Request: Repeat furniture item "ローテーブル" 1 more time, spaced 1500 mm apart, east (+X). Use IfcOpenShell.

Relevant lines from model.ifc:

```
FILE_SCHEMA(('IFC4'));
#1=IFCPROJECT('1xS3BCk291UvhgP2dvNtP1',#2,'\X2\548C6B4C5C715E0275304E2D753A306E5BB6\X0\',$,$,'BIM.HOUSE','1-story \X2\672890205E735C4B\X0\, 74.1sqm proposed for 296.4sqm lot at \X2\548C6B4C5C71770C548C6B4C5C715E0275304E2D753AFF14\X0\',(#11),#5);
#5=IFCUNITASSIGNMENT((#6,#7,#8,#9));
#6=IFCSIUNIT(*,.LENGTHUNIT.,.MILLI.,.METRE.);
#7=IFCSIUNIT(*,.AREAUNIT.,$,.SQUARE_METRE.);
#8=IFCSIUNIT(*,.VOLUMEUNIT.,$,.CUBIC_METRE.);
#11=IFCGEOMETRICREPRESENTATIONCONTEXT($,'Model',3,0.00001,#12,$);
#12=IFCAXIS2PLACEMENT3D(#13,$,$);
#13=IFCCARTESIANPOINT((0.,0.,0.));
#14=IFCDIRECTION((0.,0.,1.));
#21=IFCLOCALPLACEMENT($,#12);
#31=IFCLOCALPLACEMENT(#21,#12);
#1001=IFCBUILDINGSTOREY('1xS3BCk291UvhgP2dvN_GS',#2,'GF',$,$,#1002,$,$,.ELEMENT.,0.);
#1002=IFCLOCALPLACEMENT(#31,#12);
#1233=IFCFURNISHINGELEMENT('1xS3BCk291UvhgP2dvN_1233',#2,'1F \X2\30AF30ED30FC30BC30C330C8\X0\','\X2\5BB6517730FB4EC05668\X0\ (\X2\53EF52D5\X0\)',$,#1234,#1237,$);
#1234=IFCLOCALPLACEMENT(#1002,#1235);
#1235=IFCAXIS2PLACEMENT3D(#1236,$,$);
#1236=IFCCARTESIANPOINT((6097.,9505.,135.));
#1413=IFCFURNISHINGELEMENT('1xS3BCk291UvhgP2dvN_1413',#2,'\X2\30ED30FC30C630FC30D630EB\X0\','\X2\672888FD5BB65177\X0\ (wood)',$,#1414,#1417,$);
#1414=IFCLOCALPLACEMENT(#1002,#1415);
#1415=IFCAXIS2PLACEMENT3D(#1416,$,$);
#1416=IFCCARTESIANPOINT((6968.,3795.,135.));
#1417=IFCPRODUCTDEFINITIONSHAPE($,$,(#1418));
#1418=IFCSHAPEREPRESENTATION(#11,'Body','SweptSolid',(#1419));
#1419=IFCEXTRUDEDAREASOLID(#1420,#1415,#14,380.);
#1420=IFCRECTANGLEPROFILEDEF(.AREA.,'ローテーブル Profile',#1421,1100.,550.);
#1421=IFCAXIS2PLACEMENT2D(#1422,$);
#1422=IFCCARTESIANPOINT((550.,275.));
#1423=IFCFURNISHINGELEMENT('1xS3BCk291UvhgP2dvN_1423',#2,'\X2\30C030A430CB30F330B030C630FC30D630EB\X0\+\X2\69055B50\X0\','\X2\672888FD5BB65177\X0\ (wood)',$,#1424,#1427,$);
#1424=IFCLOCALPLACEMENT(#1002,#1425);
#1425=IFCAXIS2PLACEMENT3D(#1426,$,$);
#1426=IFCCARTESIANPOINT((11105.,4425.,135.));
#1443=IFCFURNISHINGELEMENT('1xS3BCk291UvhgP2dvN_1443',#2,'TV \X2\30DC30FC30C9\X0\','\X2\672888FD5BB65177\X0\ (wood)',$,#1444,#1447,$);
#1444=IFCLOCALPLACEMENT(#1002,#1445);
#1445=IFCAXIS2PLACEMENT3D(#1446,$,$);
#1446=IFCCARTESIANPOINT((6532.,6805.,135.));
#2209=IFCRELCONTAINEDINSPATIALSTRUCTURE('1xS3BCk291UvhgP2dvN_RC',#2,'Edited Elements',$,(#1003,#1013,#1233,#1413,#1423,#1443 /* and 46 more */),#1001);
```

```python
import numpy as np
import ifcopenshell
import ifcopenshell.api.geometry
import ifcopenshell.api.root
import ifcopenshell.util.element
import ifcopenshell.util.placement
import ifcopenshell.util.unit

model = ifcopenshell.open("model.ifc")
unit_scale = ifcopenshell.util.unit.calculate_unit_scale(model)


def reuse_history(source, copy):
    """copy_class also copies each property set's owner history, people and application; keep the originals."""
    for rel in copy.IsDefinedBy:
        if rel.is_a("IfcRelDefinesByProperties") and (history := rel.RelatingPropertyDefinition.OwnerHistory):
            rel.RelatingPropertyDefinition.OwnerHistory = source.OwnerHistory
            ifcopenshell.util.element.remove_deep2(model, history)


source = model.by_guid("1xS3BCk291UvhgP2dvN_1413")
base = ifcopenshell.util.placement.get_local_placement(source.ObjectPlacement)
step = np.array([1.0, 0.0, 0.0]) * 1.5 / unit_scale

for i in range(1, 2):
    copy = ifcopenshell.api.root.copy_class(model, product=source)
    copy.Representation = ifcopenshell.util.element.copy_deep(
        model, source.Representation, exclude=["IfcGeometricRepresentationContext", "IfcRepresentationMap"]
    )
    reuse_history(source, copy)
    matrix = base.copy()
    matrix[:3, 3] += i * step
    print("added at", matrix[:3, 3].round(3) + 0.0)
    ifcopenshell.api.geometry.edit_object_placement(model, product=copy, matrix=matrix, is_si=False)

model.write("model-out.ifc")
```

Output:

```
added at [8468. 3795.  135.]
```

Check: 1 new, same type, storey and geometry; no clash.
